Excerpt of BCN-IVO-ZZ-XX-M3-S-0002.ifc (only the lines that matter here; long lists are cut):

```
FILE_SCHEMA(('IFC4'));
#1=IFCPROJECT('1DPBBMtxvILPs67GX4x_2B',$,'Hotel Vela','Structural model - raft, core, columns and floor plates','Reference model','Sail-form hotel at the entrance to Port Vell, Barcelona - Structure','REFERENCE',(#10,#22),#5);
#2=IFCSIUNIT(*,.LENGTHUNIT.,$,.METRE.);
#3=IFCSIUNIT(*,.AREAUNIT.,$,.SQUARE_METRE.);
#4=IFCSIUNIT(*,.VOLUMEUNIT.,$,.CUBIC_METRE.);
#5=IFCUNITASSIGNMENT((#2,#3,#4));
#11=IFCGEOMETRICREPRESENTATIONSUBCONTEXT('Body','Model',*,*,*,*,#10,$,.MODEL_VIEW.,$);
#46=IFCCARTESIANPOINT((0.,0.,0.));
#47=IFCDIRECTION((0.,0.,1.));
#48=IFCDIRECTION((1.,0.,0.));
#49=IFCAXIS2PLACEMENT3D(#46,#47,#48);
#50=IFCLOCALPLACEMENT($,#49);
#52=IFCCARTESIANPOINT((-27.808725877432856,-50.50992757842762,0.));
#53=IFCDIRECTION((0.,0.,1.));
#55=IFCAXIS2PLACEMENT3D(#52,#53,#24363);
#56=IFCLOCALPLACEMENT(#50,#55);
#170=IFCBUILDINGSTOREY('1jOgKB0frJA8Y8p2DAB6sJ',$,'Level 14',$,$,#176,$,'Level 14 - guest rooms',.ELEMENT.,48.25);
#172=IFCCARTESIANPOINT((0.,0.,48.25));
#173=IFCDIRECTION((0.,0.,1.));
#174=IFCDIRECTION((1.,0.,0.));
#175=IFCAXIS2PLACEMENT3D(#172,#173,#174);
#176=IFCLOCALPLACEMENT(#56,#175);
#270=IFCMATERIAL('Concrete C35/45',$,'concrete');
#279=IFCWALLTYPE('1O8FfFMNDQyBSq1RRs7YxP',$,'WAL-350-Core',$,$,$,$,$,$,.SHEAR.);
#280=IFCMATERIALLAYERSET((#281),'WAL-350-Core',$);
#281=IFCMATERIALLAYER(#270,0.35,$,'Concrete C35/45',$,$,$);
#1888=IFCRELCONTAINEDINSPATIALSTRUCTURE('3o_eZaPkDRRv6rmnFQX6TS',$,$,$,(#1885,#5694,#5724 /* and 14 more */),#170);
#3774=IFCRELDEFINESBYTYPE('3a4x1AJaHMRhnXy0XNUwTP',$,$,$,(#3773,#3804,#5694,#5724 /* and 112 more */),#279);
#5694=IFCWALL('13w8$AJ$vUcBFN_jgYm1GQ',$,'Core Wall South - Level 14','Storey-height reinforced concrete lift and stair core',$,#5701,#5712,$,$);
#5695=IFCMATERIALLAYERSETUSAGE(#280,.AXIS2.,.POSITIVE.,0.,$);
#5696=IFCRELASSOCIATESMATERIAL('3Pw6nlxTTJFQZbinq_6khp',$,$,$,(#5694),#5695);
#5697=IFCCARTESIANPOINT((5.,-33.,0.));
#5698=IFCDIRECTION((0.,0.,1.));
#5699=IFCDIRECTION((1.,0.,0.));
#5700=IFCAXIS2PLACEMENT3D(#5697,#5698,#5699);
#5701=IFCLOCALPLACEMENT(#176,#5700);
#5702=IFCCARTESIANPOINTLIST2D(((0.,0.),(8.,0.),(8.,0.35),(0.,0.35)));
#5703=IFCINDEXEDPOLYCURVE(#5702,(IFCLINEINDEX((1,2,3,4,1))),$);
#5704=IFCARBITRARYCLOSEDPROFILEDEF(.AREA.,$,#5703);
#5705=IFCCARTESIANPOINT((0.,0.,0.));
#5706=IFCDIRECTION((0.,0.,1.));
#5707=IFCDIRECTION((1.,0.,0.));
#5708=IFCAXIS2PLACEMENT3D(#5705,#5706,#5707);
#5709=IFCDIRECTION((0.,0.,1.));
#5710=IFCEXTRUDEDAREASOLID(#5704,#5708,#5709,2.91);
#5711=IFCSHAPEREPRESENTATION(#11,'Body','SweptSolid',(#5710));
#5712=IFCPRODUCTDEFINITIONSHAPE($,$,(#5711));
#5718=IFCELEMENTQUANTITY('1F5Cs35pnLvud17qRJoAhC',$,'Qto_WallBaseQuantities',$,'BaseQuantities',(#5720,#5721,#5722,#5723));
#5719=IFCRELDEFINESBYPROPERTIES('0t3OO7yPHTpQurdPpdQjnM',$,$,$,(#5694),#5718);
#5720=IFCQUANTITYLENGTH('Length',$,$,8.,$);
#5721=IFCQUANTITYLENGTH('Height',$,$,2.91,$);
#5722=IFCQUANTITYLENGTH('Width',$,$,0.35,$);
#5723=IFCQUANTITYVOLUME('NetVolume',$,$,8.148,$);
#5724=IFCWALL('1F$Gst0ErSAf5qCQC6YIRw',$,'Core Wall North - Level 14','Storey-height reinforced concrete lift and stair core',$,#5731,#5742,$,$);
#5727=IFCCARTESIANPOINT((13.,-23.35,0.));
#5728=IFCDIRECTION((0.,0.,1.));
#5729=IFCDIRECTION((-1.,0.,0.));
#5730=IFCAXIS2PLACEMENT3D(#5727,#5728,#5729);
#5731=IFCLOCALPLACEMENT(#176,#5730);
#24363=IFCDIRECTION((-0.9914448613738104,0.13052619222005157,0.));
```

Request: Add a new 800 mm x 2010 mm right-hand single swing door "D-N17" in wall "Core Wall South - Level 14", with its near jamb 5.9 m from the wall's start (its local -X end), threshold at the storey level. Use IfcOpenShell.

```python
import numpy as np
import ifcopenshell
import ifcopenshell.api.feature
import ifcopenshell.api.geometry
import ifcopenshell.api.pset
import ifcopenshell.api.root
import ifcopenshell.api.spatial
import ifcopenshell.geom
import ifcopenshell.util.element
import ifcopenshell.util.placement
import ifcopenshell.util.representation
import ifcopenshell.util.shape
import ifcopenshell.util.unit

model = ifcopenshell.open("BCN-IVO-ZZ-XX-M3-S-0002.ifc")
unit_scale = ifcopenshell.util.unit.calculate_unit_scale(model)
volume_scale = ifcopenshell.util.unit.calculate_unit_scale(model, "VOLUMEUNIT")
settings = ifcopenshell.geom.settings()


def volume(element):
    """Net volume in cubic metres, openings subtracted."""
    shape = ifcopenshell.geom.create_shape(settings, element)
    return ifcopenshell.util.shape.get_volume(shape.geometry)


wall = model.by_guid("13w8$AJ$vUcBFN_jgYm1GQ")
storey = ifcopenshell.util.element.get_container(wall, ifc_class="IfcBuildingStorey")
context = ifcopenshell.util.representation.get_context(model, "Model", "Body", "MODEL_VIEW")
before = volume(wall)

width, height, from_end, sill = 0.8, 2.01, 5.9, 0.0  # metres

# The wall runs along its own X axis, and the end named is its -X end.
wall_shape = ifcopenshell.geom.create_shape(settings, wall)
x, y, z = ifcopenshell.util.shape.get_vertices(wall_shape.geometry).T
start = x.min() + from_end
face, thickness = float(y.min()), float(y.max() - y.min())
wall_matrix = ifcopenshell.util.placement.get_local_placement(wall.ObjectPlacement)
level = ifcopenshell.util.placement.get_local_placement(storey.ObjectPlacement)[2, 3]


def in_wall(x, y):
    """Placement at x, y metres in the wall's axes, at sill height."""
    matrix = wall_matrix.copy()
    matrix[:, 3] = wall_matrix @ np.array([x / unit_scale, y / unit_scale, 0.0, 1.0])
    matrix[2, 3] = level + sill / unit_scale
    return matrix


# Opening: a box that overshoots both wall faces by 50 mm.
opening = ifcopenshell.api.root.create_entity(model, ifc_class="IfcOpeningElement", predefined_type="OPENING")
box = ifcopenshell.api.geometry.add_wall_representation(
    model, context=context, length=width, height=height, thickness=thickness + 0.1
)
ifcopenshell.api.geometry.assign_representation(model, product=opening, representation=box)
ifcopenshell.api.geometry.edit_object_placement(model, product=opening, matrix=in_wall(start, face - 0.05), is_si=False)
ifcopenshell.api.feature.add_feature(model, feature=opening, element=wall)

door = ifcopenshell.api.root.create_entity(model, ifc_class="IfcDoor", name="D-N17", predefined_type="DOOR")
door.OverallWidth, door.OverallHeight = width / unit_scale, height / unit_scale
door.OperationType = "SINGLE_SWING_RIGHT"
body = ifcopenshell.api.geometry.add_door_representation(
    model,
    context=context,
    overall_width=door.OverallWidth,
    overall_height=door.OverallHeight,
    operation_type="SINGLE_SWING_RIGHT",
    lining_properties={"LiningDepth": thickness / unit_scale, "ThresholdDepth": thickness / unit_scale},
)
ifcopenshell.api.geometry.assign_representation(model, product=door, representation=body)
ifcopenshell.api.spatial.assign_container(model, products=[door], relating_structure=storey)
ifcopenshell.api.feature.add_filling(model, opening=opening, element=door)

# The lining spans the wall, so the door starts at the wall face.
ifcopenshell.api.geometry.edit_object_placement(model, product=door, matrix=in_wall(start, face), is_si=False)

after = volume(wall)

# Update the wall's stored quantities.
qto = model.by_id(ifcopenshell.util.element.get_pset(wall, "Qto_WallBaseQuantities", should_inherit=False)["id"])
ifcopenshell.api.pset.edit_qto(model, qto=qto, properties={"NetVolume": after / volume_scale})

print(f"wall volume {before:.3f} -> {after:.3f} m3")

model.write("BCN-IVO-ZZ-XX-M3-S-0002_updated.ifc")
```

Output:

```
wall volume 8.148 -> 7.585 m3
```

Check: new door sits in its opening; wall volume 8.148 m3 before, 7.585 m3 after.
